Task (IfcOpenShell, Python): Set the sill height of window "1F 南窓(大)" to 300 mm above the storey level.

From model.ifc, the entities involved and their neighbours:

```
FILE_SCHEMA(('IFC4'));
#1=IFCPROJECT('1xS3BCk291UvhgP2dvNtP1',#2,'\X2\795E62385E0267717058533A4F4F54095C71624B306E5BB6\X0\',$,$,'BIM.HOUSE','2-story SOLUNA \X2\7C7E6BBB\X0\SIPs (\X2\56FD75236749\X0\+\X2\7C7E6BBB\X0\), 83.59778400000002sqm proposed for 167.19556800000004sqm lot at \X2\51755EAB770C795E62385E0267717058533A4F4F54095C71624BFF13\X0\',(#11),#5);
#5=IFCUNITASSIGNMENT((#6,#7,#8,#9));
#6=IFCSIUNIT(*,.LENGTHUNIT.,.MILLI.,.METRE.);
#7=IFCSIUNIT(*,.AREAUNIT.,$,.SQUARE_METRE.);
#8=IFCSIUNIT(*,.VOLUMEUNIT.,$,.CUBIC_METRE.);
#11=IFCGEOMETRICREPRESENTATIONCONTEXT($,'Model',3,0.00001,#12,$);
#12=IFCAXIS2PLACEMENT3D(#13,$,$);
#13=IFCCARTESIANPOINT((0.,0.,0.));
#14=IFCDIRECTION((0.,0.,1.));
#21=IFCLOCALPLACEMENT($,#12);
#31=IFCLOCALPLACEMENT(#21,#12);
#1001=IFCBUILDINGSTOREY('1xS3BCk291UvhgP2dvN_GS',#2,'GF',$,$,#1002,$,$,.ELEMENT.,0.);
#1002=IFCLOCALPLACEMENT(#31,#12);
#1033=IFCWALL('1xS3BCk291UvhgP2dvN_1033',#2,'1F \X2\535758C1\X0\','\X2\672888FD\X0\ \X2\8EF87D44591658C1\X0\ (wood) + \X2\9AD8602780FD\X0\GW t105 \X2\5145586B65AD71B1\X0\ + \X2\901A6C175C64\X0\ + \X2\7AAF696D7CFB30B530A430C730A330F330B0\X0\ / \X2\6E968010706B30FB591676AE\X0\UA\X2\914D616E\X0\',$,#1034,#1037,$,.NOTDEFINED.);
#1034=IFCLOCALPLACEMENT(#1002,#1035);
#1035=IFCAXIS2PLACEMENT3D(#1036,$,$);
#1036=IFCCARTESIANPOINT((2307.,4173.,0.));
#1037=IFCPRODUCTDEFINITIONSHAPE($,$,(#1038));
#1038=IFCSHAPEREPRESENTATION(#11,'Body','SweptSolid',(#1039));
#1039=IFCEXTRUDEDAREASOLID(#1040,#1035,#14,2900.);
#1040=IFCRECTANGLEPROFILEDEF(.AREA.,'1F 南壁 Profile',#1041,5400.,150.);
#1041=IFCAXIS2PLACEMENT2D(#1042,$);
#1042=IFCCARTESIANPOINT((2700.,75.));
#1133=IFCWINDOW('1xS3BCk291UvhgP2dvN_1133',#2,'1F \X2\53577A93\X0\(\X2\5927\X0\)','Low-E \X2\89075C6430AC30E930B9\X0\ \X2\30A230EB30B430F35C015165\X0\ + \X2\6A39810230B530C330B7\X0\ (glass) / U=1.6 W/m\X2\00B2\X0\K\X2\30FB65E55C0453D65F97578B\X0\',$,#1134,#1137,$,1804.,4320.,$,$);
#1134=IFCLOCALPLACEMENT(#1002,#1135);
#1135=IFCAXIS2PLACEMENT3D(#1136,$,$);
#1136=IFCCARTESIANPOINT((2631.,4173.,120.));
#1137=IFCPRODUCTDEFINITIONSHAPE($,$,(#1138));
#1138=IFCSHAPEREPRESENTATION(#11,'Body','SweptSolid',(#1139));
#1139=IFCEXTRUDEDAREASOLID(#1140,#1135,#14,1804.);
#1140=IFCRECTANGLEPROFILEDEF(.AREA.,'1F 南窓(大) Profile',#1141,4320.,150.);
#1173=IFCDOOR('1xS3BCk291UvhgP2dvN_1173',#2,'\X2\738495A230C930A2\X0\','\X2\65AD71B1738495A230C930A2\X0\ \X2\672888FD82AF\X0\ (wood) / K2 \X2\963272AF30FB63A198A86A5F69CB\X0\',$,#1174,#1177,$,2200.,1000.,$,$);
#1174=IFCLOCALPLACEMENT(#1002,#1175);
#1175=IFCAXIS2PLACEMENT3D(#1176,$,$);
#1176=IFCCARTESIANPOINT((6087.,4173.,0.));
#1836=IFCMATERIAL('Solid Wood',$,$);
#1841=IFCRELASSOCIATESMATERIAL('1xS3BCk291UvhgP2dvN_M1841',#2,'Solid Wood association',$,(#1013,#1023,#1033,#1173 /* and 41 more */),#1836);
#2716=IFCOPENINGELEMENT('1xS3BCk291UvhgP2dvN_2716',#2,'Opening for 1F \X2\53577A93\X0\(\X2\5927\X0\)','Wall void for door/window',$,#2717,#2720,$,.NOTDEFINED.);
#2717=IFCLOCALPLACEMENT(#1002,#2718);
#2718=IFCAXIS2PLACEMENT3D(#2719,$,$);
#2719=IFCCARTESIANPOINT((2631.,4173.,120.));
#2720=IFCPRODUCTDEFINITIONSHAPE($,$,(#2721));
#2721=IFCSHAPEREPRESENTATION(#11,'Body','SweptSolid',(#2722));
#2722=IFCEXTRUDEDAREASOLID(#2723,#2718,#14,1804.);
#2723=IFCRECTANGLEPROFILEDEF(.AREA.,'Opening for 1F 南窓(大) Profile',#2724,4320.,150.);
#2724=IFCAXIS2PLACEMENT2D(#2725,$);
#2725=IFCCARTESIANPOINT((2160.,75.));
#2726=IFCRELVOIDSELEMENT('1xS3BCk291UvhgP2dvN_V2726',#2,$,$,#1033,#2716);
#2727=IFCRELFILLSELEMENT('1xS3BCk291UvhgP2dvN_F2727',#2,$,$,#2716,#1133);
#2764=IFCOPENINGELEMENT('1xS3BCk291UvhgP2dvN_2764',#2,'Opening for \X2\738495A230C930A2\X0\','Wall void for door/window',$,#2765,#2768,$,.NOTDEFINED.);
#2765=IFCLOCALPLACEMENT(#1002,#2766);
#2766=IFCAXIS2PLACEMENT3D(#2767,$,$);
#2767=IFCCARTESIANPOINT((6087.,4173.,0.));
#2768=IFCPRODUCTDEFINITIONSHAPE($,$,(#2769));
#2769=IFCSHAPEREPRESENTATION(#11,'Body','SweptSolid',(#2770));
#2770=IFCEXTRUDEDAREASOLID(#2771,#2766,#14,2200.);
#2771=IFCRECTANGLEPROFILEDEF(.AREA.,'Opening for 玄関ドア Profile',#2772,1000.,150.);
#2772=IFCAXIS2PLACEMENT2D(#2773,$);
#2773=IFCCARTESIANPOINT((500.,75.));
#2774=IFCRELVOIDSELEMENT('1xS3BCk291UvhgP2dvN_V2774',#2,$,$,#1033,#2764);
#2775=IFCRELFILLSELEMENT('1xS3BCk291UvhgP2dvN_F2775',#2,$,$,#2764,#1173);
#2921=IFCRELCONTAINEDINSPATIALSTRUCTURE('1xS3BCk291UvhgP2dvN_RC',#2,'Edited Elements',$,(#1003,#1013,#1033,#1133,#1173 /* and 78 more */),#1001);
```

```python
import numpy as np
import ifcopenshell
import ifcopenshell.api.geometry
import ifcopenshell.geom
import ifcopenshell.util.element
import ifcopenshell.util.placement
import ifcopenshell.util.shape
import ifcopenshell.util.unit

model = ifcopenshell.open("model.ifc")
unit_scale = ifcopenshell.util.unit.calculate_unit_scale(model)

window = model.by_guid("1xS3BCk291UvhgP2dvN_1133")
opening = window.FillsVoids[0].RelatingOpeningElement
storey = ifcopenshell.util.element.get_container(window, ifc_class="IfcBuildingStorey")
level = ifcopenshell.util.placement.get_local_placement(storey.ObjectPlacement)[2, 3]

# The opening's origin need not be at the sill, so measure its lowest point.
shape = ifcopenshell.geom.create_shape(ifcopenshell.geom.settings(), opening)
bottom = ifcopenshell.util.shape.get_shape_bottom_elevation(shape, shape.geometry) / unit_scale
dz = level + 300.0 - bottom

shift = np.array([0.0, 0.0, dz])
# The window is not placed relative to its opening, so move both.
for product in (opening, window):
    matrix = ifcopenshell.util.placement.get_local_placement(product.ObjectPlacement)
    matrix[:3, 3] += shift
    ifcopenshell.api.geometry.edit_object_placement(model, product=product, matrix=matrix, is_si=False)

print(f"moved by {dz * unit_scale:+.3f} m")

model.write("model_v2.ifc")
```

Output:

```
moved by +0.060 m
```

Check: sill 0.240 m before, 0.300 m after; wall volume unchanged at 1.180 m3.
